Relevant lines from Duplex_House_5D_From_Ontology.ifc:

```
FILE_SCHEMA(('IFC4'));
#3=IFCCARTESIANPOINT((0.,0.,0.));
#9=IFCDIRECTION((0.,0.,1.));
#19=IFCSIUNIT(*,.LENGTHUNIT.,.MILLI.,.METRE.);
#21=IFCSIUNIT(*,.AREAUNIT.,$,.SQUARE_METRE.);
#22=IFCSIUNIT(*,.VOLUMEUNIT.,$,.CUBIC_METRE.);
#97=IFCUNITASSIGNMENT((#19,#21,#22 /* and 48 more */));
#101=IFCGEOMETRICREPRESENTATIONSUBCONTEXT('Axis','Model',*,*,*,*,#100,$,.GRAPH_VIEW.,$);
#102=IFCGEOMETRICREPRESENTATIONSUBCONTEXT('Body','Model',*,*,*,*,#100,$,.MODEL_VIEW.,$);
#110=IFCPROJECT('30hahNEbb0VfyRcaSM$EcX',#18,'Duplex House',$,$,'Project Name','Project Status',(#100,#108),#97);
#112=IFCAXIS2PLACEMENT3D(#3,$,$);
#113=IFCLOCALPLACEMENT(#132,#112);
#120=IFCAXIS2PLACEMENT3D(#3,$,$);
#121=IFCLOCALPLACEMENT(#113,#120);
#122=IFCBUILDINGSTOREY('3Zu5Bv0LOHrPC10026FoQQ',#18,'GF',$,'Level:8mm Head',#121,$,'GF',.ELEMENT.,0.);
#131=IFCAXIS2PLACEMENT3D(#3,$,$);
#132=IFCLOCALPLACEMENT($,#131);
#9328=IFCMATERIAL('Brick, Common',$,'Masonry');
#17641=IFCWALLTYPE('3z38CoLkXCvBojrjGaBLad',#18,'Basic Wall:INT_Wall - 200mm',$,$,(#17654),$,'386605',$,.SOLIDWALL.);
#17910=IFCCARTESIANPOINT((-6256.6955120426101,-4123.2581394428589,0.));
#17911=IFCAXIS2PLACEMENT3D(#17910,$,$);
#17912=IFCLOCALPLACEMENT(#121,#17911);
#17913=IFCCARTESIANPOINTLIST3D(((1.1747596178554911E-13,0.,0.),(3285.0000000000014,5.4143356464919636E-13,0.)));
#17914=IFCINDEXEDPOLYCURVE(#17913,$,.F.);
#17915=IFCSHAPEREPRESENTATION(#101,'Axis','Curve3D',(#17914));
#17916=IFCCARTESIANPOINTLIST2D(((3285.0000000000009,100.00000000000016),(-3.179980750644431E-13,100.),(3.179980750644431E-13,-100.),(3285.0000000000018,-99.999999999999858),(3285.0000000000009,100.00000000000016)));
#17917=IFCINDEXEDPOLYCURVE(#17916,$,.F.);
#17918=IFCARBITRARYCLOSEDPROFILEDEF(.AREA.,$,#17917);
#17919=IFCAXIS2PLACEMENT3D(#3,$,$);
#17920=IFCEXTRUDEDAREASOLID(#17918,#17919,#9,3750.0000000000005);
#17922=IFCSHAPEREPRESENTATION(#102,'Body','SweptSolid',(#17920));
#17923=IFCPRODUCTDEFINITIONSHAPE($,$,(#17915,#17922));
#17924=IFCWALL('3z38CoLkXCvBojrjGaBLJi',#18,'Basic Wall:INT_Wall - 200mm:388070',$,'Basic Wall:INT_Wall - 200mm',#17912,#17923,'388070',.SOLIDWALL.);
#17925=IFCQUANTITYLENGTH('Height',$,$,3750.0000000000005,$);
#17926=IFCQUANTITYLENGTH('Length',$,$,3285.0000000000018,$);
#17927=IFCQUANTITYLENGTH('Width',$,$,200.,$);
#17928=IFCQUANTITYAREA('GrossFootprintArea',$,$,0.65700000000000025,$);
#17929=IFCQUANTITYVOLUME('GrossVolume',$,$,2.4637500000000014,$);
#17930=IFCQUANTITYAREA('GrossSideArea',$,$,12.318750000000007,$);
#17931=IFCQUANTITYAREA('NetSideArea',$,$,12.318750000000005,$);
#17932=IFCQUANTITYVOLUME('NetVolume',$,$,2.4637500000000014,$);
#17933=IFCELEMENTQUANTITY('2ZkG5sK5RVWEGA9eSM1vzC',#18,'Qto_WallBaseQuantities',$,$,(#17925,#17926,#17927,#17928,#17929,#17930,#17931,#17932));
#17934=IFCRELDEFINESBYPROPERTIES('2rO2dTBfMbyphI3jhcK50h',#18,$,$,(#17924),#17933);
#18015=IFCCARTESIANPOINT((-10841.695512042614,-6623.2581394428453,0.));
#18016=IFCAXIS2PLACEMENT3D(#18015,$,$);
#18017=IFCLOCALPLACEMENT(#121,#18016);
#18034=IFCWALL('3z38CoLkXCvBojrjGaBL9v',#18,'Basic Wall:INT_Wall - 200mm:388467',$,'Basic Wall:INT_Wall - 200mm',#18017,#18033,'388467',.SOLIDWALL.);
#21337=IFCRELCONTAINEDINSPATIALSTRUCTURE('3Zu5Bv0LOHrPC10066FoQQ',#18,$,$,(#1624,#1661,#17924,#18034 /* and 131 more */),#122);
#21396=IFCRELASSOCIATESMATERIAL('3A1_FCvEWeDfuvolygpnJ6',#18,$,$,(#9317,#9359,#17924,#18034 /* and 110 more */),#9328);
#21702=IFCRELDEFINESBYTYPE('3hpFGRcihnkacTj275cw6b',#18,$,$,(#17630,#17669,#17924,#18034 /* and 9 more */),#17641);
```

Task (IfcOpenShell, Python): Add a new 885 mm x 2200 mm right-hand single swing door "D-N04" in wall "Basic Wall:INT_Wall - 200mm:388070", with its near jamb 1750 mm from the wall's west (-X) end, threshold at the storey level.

```python
import numpy as np
import ifcopenshell
import ifcopenshell.api.feature
import ifcopenshell.api.geometry
import ifcopenshell.api.pset
import ifcopenshell.api.root
import ifcopenshell.api.spatial
import ifcopenshell.geom
import ifcopenshell.util.element
import ifcopenshell.util.placement
import ifcopenshell.util.representation
import ifcopenshell.util.shape
import ifcopenshell.util.unit

model = ifcopenshell.open("Duplex_House_5D_From_Ontology.ifc")
unit_scale = ifcopenshell.util.unit.calculate_unit_scale(model)
area_scale = ifcopenshell.util.unit.calculate_unit_scale(model, "AREAUNIT")
volume_scale = ifcopenshell.util.unit.calculate_unit_scale(model, "VOLUMEUNIT")
settings = ifcopenshell.geom.settings()


def volume(element):
    """Net volume in cubic metres, openings subtracted."""
    shape = ifcopenshell.geom.create_shape(settings, element)
    return ifcopenshell.util.shape.get_volume(shape.geometry)


wall = model.by_guid("3z38CoLkXCvBojrjGaBLJi")
storey = ifcopenshell.util.element.get_container(wall, ifc_class="IfcBuildingStorey")
context = ifcopenshell.util.representation.get_context(model, "Model", "Body", "MODEL_VIEW")
before = volume(wall)

width, height, from_end, sill = 0.885, 2.2, 1.75, 0.0  # metres

# The wall runs along its own X axis, and the end named is its -X end.
wall_shape = ifcopenshell.geom.create_shape(settings, wall)
x, y, z = ifcopenshell.util.shape.get_vertices(wall_shape.geometry).T
start = x.min() + from_end
face, thickness = float(y.min()), float(y.max() - y.min())
wall_matrix = ifcopenshell.util.placement.get_local_placement(wall.ObjectPlacement)
level = ifcopenshell.util.placement.get_local_placement(storey.ObjectPlacement)[2, 3]


def in_wall(x, y):
    """Placement at x, y metres in the wall's axes, at sill height."""
    matrix = wall_matrix.copy()
    matrix[:, 3] = wall_matrix @ np.array([x / unit_scale, y / unit_scale, 0.0, 1.0])
    matrix[2, 3] = level + sill / unit_scale
    return matrix


# Opening: a box that overshoots both wall faces by 50 mm.
opening = ifcopenshell.api.root.create_entity(model, ifc_class="IfcOpeningElement", predefined_type="OPENING")
box = ifcopenshell.api.geometry.add_wall_representation(
    model, context=context, length=width, height=height, thickness=thickness + 0.1
)
ifcopenshell.api.geometry.assign_representation(model, product=opening, representation=box)
ifcopenshell.api.geometry.edit_object_placement(model, product=opening, matrix=in_wall(start, face - 0.05), is_si=False)
ifcopenshell.api.feature.add_feature(model, feature=opening, element=wall)

door = ifcopenshell.api.root.create_entity(model, ifc_class="IfcDoor", name="D-N04", predefined_type="DOOR")
door.OverallWidth, door.OverallHeight = width / unit_scale, height / unit_scale
door.OperationType = "SINGLE_SWING_RIGHT"
body = ifcopenshell.api.geometry.add_door_representation(
    model,
    context=context,
    overall_width=door.OverallWidth,
    overall_height=door.OverallHeight,
    operation_type="SINGLE_SWING_RIGHT",
    lining_properties={"LiningDepth": thickness / unit_scale, "ThresholdDepth": thickness / unit_scale},
)
ifcopenshell.api.geometry.assign_representation(model, product=door, representation=body)
ifcopenshell.api.spatial.assign_container(model, products=[door], relating_structure=storey)
ifcopenshell.api.feature.add_filling(model, opening=opening, element=door)

# The lining spans the wall, so the door starts at the wall face.
ifcopenshell.api.geometry.edit_object_placement(model, product=door, matrix=in_wall(start, face), is_si=False)

after = volume(wall)

# Update the wall's stored quantities.
qto = model.by_id(ifcopenshell.util.element.get_pset(wall, "Qto_WallBaseQuantities", should_inherit=False)["id"])
ifcopenshell.api.pset.edit_qto(model, qto=qto, properties={
    "NetSideArea": after / thickness / area_scale,
    "NetVolume": after / volume_scale,
})

print(f"wall volume {before:.3f} -> {after:.3f} m3")

model.write("Duplex_House_5D_From_Ontology-out.ifc")
```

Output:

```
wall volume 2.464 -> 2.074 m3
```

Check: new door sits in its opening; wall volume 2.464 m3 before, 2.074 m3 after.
